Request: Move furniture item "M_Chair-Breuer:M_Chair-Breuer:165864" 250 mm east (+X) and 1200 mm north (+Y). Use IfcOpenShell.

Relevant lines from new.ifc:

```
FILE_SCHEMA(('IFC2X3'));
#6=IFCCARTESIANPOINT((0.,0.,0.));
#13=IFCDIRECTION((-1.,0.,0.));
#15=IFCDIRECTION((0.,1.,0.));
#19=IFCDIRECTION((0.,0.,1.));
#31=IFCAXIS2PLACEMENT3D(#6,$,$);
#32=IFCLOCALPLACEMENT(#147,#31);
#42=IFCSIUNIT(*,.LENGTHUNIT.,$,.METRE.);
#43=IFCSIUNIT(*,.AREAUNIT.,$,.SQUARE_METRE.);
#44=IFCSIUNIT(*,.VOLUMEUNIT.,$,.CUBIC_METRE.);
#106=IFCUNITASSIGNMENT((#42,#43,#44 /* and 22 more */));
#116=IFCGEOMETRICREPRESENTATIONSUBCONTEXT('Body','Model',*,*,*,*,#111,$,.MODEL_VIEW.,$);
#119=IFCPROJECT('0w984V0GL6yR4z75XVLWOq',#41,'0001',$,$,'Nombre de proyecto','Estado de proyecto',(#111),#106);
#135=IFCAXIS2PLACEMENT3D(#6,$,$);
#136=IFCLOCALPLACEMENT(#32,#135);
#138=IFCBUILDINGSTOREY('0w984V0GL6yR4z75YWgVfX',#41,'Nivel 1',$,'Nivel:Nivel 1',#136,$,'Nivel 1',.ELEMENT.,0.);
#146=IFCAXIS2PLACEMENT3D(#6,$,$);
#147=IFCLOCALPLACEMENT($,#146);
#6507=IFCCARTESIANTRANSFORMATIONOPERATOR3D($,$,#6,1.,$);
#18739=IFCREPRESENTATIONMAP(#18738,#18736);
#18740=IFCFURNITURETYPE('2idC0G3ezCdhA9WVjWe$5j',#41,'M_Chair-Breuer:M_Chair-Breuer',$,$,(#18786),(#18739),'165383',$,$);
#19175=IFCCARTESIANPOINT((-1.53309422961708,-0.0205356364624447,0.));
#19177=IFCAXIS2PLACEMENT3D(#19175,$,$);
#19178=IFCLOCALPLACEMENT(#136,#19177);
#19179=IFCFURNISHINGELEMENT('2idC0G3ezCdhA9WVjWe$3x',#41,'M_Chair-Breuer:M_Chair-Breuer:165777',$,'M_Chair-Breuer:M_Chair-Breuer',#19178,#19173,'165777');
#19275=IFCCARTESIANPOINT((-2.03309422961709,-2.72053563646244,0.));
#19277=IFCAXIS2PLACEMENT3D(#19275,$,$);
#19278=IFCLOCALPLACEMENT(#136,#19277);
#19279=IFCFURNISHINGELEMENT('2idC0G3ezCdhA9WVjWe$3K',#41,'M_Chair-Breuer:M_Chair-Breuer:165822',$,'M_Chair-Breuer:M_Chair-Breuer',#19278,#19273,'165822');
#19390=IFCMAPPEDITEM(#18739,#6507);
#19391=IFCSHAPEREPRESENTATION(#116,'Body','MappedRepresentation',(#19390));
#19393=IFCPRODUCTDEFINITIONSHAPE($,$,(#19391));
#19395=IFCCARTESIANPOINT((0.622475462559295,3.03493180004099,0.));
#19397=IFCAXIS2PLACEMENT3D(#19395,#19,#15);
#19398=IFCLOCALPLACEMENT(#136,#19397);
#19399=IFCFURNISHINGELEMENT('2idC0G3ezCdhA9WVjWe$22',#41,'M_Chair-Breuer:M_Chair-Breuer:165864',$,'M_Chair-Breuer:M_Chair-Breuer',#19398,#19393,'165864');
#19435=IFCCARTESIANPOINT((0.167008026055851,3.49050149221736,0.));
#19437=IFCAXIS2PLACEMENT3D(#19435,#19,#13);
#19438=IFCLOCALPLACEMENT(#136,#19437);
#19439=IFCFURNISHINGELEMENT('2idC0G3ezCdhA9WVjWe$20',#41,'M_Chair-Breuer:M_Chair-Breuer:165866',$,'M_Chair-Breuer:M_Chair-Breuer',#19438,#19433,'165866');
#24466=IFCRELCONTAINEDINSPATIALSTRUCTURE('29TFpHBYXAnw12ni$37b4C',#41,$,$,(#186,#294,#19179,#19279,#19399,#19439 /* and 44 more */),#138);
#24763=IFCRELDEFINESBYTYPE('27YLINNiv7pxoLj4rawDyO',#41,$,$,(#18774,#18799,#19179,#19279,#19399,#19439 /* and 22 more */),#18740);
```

```python
import ifcopenshell
import ifcopenshell.api.geometry
import ifcopenshell.util.placement

model = ifcopenshell.open("new.ifc")

item = model.by_id(19399)
matrix = ifcopenshell.util.placement.get_local_placement(item.ObjectPlacement)
matrix[0, 3] += 0.25
matrix[1, 3] += 1.2
ifcopenshell.api.geometry.edit_object_placement(model, product=item, matrix=matrix, is_si=False)

print(ifcopenshell.util.placement.get_local_placement(item.ObjectPlacement).round(3) + 0.0)

model.write("new_updated.ifc")
```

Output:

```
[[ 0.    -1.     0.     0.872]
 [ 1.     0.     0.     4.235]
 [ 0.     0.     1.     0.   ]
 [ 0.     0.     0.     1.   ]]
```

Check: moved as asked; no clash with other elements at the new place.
